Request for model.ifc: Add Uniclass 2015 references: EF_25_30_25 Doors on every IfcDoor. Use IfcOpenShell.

First a look at what the model holds.

```python
import ifcopenshell

model = ifcopenshell.open("model.ifc")
print(model.schema)
print("classifications:", [c.Name for c in model.by_type("IfcClassification")])
for ifc_class in ("IfcDoor", "IfcRoof", "IfcStair", "IfcWall", "IfcWindow"):
    print(ifc_class, len(model.by_type(ifc_class)))
```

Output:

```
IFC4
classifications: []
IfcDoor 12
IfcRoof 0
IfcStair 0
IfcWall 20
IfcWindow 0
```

```python
import ifcopenshell
import ifcopenshell.api.classification

model = ifcopenshell.open("model.ifc")

system = ifcopenshell.api.classification.add_classification(model, classification="Uniclass 2015")

codes = {
    "IfcDoor": ("EF_25_30_25", "Doors"),
}
for ifc_class, (code, name) in codes.items():
    products = model.by_type(ifc_class)
    ifcopenshell.api.classification.add_reference(
        model, products=products, classification=system, identification=code, name=name
    )
    print(code, len(products))

model.write("model_updated.ifc")
```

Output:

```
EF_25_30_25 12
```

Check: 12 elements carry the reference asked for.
